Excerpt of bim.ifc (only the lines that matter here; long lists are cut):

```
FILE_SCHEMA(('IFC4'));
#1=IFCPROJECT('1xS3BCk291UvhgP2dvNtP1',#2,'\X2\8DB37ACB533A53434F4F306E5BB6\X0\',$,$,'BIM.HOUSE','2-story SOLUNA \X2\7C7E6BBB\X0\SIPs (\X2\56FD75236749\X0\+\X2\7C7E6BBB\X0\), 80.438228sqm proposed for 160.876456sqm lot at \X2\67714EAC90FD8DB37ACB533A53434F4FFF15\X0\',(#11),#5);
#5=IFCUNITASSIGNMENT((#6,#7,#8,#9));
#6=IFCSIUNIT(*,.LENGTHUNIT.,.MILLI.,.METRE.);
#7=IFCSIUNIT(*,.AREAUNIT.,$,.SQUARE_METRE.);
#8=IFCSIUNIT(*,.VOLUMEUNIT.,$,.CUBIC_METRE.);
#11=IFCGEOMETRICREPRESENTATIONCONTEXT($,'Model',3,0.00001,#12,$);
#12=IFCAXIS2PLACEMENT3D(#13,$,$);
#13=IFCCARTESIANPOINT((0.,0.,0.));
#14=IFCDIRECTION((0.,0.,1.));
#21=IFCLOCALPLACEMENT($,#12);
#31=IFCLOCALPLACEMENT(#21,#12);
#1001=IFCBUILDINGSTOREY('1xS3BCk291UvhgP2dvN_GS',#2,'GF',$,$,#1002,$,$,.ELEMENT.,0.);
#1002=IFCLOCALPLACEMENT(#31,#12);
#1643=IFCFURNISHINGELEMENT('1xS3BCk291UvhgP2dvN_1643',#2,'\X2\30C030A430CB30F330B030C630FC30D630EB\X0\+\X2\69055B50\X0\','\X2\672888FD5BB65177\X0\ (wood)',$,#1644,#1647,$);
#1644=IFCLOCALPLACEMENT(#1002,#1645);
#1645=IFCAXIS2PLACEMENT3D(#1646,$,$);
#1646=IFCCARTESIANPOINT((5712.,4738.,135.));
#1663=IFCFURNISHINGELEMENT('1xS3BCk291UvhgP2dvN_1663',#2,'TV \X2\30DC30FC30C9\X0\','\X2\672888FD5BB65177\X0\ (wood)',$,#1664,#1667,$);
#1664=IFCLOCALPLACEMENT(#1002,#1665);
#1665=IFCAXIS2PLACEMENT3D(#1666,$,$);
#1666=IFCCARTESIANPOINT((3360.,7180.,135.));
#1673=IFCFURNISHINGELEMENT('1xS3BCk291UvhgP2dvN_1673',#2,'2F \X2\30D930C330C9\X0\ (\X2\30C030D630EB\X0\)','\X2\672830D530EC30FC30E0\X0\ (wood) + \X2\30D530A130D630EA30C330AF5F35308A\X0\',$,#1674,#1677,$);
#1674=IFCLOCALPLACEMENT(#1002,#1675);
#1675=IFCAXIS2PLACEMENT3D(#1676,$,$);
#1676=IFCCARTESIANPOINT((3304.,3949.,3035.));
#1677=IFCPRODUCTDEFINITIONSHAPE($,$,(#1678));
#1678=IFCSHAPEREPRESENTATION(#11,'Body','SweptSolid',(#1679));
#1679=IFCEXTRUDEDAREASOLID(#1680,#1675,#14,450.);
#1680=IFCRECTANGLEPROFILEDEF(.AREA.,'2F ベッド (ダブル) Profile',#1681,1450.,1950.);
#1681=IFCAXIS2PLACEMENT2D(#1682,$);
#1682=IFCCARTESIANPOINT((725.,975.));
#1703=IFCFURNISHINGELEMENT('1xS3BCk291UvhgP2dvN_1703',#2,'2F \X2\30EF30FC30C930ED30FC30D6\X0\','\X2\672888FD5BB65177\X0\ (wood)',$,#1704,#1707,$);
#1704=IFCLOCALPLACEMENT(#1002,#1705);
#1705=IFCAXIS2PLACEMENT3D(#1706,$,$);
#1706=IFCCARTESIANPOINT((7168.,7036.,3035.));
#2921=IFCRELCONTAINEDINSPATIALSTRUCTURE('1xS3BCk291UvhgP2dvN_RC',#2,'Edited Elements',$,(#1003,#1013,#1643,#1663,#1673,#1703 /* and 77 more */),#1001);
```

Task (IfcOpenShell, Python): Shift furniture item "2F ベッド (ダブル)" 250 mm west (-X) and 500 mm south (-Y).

```python
import ifcopenshell
import ifcopenshell.api.geometry
import ifcopenshell.util.placement
import ifcopenshell.util.unit

model = ifcopenshell.open("bim.ifc")
unit_scale = ifcopenshell.util.unit.calculate_unit_scale(model)

item = model.by_guid("1xS3BCk291UvhgP2dvN_1673")
matrix = ifcopenshell.util.placement.get_local_placement(item.ObjectPlacement)
matrix[0, 3] -= 0.25 / unit_scale
matrix[1, 3] -= 0.5 / unit_scale
ifcopenshell.api.geometry.edit_object_placement(model, product=item, matrix=matrix, is_si=False)

print(ifcopenshell.util.placement.get_local_placement(item.ObjectPlacement).round(3) + 0.0)

model.write("bim_v2.ifc")
```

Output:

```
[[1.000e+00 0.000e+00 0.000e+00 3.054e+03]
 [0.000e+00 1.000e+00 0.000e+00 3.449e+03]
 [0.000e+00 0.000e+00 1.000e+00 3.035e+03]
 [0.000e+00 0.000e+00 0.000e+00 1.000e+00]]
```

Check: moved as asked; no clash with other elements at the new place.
